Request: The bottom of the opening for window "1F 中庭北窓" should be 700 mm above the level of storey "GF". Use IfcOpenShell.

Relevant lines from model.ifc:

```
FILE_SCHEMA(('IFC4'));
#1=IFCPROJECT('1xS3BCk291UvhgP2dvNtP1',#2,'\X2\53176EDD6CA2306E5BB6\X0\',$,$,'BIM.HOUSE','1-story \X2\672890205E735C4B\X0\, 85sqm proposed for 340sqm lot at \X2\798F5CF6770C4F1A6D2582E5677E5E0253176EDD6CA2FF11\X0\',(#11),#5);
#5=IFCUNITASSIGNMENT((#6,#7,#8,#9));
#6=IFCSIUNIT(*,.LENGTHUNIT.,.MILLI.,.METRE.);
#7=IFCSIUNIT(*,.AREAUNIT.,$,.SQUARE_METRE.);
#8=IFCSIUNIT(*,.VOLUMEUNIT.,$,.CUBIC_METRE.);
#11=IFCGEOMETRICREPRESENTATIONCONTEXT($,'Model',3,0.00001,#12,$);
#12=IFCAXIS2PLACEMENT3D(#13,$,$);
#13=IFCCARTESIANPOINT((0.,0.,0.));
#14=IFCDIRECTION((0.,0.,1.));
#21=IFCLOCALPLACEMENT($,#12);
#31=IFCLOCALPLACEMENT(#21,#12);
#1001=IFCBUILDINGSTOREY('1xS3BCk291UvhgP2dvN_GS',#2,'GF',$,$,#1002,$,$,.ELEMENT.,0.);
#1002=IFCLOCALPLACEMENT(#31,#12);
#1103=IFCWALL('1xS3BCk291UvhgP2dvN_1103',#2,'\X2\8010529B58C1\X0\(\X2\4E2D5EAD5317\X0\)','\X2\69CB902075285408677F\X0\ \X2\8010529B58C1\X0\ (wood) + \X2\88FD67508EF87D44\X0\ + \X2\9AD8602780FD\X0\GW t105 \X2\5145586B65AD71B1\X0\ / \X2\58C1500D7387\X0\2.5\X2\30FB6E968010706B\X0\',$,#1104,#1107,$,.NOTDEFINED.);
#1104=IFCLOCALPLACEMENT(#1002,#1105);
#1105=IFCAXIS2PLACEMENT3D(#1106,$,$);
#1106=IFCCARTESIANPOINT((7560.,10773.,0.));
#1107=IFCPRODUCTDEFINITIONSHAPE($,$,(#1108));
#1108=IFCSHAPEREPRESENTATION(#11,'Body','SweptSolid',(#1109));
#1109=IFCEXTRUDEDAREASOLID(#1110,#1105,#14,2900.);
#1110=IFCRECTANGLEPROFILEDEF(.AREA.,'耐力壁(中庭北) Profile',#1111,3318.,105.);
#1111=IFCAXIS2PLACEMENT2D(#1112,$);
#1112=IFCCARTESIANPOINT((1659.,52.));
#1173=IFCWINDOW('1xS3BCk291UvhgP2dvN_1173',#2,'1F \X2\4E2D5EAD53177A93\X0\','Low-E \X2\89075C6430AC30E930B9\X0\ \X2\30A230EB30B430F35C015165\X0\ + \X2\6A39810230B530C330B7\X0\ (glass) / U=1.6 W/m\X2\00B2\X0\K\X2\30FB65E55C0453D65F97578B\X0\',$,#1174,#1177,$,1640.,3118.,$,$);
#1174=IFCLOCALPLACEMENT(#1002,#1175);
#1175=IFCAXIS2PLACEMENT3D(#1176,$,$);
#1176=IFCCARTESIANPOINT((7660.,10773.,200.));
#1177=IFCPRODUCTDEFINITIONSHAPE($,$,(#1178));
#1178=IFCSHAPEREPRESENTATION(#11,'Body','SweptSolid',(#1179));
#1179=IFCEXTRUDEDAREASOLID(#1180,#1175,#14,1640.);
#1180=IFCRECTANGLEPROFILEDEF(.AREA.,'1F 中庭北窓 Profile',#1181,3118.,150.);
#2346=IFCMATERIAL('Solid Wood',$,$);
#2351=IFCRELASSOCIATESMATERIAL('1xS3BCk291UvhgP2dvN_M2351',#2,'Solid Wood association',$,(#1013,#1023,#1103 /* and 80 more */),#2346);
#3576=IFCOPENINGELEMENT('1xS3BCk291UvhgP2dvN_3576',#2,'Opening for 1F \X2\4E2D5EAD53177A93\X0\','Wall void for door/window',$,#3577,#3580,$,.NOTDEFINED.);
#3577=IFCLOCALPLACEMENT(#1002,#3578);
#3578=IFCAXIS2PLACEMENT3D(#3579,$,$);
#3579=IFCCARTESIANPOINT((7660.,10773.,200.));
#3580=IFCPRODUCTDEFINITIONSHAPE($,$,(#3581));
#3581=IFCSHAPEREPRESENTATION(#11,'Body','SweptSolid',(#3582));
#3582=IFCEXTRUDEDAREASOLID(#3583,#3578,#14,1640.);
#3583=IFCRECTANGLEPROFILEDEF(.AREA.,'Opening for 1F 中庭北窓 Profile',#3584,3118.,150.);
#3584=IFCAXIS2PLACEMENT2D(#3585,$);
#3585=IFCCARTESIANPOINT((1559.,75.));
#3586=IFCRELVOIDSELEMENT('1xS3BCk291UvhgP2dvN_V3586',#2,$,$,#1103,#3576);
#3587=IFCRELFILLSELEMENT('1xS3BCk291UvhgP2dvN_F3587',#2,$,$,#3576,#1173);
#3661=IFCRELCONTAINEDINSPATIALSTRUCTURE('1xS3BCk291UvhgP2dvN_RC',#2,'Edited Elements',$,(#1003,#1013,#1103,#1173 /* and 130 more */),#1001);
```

```python
import numpy as np
import ifcopenshell
import ifcopenshell.api.geometry
import ifcopenshell.geom
import ifcopenshell.util.element
import ifcopenshell.util.placement
import ifcopenshell.util.shape
import ifcopenshell.util.unit

model = ifcopenshell.open("model.ifc")
unit_scale = ifcopenshell.util.unit.calculate_unit_scale(model)

window = model.by_guid("1xS3BCk291UvhgP2dvN_1173")
opening = window.FillsVoids[0].RelatingOpeningElement
storey = ifcopenshell.util.element.get_container(window, ifc_class="IfcBuildingStorey")
level = ifcopenshell.util.placement.get_local_placement(storey.ObjectPlacement)[2, 3]

# The opening's origin need not be at the sill, so measure its lowest point.
shape = ifcopenshell.geom.create_shape(ifcopenshell.geom.settings(), opening)
bottom = ifcopenshell.util.shape.get_shape_bottom_elevation(shape, shape.geometry) / unit_scale
dz = level + 700.0 - bottom

shift = np.array([0.0, 0.0, dz])
# The window is not placed relative to its opening, so move both.
for product in (opening, window):
    matrix = ifcopenshell.util.placement.get_local_placement(product.ObjectPlacement)
    matrix[:3, 3] += shift
    ifcopenshell.api.geometry.edit_object_placement(model, product=product, matrix=matrix, is_si=False)

print(f"moved by {dz * unit_scale:+.3f} m")

model.write("model_updated.ifc")
```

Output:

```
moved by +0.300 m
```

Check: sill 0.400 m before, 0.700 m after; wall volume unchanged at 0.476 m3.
